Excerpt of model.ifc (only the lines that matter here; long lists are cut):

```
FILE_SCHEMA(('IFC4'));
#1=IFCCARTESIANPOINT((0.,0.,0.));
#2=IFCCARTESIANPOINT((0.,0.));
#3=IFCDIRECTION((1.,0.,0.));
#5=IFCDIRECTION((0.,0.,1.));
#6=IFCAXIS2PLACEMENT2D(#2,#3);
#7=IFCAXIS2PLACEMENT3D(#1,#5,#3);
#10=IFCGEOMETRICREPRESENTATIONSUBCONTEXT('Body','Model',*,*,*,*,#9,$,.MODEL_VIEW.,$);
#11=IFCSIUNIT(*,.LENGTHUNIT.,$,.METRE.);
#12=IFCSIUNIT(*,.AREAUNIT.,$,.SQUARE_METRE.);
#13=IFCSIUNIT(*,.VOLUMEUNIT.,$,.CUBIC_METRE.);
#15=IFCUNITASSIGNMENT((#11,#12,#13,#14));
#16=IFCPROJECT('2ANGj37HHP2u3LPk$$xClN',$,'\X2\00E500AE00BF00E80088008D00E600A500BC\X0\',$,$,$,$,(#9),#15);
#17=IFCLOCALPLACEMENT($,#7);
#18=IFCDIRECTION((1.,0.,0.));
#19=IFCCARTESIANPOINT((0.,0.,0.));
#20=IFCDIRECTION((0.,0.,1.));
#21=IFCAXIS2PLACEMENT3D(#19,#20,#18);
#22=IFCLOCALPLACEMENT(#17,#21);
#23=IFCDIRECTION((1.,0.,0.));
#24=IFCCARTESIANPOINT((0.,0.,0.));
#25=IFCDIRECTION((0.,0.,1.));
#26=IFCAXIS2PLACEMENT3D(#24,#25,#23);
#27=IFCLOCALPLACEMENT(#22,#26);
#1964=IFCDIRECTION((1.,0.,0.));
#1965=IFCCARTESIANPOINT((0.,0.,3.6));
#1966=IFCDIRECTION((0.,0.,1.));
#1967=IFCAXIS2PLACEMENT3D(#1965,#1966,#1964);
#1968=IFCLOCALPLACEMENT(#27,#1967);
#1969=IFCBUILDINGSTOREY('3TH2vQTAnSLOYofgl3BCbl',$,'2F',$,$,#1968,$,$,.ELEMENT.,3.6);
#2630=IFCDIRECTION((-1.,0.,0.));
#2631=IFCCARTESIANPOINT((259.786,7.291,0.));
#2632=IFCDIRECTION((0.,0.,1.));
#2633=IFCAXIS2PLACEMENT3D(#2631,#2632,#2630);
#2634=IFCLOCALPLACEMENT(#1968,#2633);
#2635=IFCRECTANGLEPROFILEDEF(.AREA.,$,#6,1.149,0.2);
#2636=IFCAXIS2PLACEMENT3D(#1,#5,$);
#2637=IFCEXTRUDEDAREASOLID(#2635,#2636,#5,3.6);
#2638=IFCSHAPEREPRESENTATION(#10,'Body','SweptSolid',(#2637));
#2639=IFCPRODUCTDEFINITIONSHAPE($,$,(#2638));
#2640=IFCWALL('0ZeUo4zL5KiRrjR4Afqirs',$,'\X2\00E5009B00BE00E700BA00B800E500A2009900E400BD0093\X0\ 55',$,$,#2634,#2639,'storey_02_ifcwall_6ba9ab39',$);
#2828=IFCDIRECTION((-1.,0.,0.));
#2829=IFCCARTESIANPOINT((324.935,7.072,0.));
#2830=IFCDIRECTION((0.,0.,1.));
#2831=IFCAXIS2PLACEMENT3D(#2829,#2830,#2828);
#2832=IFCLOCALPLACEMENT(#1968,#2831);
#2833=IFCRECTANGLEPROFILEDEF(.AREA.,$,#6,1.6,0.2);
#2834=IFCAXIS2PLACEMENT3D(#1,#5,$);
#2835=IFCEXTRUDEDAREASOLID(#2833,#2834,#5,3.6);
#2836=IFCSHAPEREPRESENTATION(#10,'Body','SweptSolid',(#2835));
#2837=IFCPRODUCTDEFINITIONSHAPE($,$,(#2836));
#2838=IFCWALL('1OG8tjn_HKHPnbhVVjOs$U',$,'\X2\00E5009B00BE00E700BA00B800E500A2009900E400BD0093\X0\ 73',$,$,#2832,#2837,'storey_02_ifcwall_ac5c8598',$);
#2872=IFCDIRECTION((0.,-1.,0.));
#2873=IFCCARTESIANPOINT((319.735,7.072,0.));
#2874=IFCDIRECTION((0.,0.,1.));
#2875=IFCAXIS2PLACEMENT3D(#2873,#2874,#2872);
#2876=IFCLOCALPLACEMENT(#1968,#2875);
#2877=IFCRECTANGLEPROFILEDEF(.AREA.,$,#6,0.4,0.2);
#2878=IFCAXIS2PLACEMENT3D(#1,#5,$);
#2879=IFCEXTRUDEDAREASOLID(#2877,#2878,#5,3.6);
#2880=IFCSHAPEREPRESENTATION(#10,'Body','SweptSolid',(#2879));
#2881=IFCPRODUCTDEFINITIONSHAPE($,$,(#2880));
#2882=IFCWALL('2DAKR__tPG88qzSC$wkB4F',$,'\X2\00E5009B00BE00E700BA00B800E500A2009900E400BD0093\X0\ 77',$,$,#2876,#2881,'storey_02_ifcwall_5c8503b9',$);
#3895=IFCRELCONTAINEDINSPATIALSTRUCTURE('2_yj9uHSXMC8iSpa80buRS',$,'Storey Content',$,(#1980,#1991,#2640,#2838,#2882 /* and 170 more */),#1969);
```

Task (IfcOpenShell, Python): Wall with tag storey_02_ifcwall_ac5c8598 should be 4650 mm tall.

```python
import ifcopenshell
import ifcopenshell.geom
import ifcopenshell.util.representation
import ifcopenshell.util.shape
import ifcopenshell.util.unit

model = ifcopenshell.open("model.ifc")
unit_scale = ifcopenshell.util.unit.calculate_unit_scale(model)
settings = ifcopenshell.geom.settings()


def volume(element):
    """Net volume in cubic metres, openings subtracted."""
    shape = ifcopenshell.geom.create_shape(settings, element)
    return ifcopenshell.util.shape.get_volume(shape.geometry)


wall = model.by_guid("1OG8tjn_HKHPnbhVVjOs$U")
before = volume(wall)

body = ifcopenshell.util.representation.get_representation(wall, "Model", "Body")
solid = body.Items[0]
old_height = solid.Depth
solid.Depth = 4.65 / unit_scale
after = volume(wall)

print(f"height {old_height:g} -> {solid.Depth:g}, volume {before:.3f} -> {after:.3f} m3")

model.write("model-out.ifc")
```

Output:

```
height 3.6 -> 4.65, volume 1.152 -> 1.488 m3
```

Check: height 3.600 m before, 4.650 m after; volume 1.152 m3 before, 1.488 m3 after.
